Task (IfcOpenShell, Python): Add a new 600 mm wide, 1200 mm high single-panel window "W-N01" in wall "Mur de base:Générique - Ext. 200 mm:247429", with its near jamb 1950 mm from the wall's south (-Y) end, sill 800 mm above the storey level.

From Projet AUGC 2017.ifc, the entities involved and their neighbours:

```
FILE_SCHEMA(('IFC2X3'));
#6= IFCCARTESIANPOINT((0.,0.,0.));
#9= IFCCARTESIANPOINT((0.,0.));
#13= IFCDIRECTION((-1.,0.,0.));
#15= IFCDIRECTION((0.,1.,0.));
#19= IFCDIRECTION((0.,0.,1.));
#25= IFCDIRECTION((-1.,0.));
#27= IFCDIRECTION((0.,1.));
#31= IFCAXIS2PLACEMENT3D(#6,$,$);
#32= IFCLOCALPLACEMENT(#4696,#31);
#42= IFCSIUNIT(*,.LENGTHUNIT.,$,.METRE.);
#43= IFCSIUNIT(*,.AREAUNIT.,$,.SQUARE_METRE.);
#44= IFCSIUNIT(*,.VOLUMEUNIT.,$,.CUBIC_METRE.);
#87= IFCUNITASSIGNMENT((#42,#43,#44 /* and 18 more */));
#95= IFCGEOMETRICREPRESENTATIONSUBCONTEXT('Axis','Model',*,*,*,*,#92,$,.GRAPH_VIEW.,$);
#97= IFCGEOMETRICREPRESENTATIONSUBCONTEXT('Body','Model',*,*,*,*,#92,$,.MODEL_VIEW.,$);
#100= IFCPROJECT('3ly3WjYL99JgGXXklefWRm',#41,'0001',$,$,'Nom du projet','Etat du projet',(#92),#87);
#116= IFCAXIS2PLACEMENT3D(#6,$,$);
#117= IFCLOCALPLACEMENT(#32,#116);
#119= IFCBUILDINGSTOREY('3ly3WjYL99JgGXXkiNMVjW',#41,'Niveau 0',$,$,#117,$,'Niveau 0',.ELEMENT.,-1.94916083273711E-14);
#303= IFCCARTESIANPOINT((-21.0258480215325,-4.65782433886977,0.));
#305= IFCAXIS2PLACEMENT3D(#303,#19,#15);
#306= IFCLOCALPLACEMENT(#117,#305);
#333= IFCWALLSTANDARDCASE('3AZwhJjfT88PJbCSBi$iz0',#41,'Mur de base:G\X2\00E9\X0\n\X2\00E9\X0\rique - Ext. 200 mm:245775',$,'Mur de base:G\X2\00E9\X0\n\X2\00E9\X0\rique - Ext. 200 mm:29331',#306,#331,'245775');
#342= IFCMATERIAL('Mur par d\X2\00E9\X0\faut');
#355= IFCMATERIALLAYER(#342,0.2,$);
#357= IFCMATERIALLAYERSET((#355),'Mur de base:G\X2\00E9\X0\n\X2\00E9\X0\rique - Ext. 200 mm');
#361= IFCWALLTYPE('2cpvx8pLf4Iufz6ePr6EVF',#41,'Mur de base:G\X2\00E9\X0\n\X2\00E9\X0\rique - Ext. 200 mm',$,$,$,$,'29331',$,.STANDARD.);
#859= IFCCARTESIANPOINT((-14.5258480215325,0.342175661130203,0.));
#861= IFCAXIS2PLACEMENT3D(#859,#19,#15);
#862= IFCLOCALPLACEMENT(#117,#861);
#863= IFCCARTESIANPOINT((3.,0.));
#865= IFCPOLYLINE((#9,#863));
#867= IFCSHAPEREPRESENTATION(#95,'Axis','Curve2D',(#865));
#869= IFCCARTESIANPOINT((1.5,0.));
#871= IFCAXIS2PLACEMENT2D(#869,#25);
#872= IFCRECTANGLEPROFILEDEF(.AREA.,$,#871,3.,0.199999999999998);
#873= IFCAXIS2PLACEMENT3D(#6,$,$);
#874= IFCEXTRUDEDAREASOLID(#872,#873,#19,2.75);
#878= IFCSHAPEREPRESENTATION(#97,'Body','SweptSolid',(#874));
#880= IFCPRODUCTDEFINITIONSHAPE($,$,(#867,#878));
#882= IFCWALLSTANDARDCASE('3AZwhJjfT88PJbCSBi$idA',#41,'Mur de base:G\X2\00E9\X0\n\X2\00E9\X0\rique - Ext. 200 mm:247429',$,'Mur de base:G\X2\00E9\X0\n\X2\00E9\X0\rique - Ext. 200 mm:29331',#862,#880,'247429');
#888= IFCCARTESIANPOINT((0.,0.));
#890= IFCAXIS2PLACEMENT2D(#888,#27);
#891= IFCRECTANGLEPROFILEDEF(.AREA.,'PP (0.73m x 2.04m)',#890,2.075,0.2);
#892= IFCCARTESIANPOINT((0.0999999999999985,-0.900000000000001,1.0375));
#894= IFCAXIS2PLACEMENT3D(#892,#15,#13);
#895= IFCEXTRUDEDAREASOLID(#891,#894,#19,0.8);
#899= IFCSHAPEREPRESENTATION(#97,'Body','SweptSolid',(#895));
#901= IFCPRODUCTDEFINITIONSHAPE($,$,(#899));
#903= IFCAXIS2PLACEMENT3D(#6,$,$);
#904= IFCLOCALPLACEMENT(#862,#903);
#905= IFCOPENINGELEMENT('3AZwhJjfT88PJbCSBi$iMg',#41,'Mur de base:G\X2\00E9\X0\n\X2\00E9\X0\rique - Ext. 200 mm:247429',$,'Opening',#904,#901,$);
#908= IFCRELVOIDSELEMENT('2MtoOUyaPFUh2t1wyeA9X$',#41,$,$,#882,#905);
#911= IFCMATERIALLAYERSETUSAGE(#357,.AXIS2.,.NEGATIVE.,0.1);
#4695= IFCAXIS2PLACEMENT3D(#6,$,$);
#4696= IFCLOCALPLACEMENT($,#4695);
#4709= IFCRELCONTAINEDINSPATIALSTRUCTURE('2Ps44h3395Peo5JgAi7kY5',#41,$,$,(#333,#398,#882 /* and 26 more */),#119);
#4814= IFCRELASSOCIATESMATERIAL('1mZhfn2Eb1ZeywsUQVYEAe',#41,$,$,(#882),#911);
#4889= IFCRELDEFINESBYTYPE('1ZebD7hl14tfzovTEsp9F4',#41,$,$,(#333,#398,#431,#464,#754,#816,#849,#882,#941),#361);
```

```python
import numpy as np
import ifcopenshell
import ifcopenshell.api.feature
import ifcopenshell.api.geometry
import ifcopenshell.api.root
import ifcopenshell.api.spatial
import ifcopenshell.api.type
import ifcopenshell.geom
import ifcopenshell.util.element
import ifcopenshell.util.placement
import ifcopenshell.util.representation
import ifcopenshell.util.shape
import ifcopenshell.util.unit

model = ifcopenshell.open("Projet AUGC 2017.ifc")
unit_scale = ifcopenshell.util.unit.calculate_unit_scale(model)
settings = ifcopenshell.geom.settings()


def volume(element):
    """Net volume in cubic metres, openings subtracted."""
    shape = ifcopenshell.geom.create_shape(settings, element)
    return ifcopenshell.util.shape.get_volume(shape.geometry)


wall = model.by_guid("3AZwhJjfT88PJbCSBi$idA")
storey = ifcopenshell.util.element.get_container(wall, ifc_class="IfcBuildingStorey")
context = ifcopenshell.util.representation.get_context(model, "Model", "Body", "MODEL_VIEW")
before = volume(wall)

width, height, from_end, sill = 0.6, 1.2, 1.95, 0.8  # metres

# The wall runs along its own X axis, and the end named is its -X end.
wall_shape = ifcopenshell.geom.create_shape(settings, wall)
x, y, z = ifcopenshell.util.shape.get_vertices(wall_shape.geometry).T
start = x.min() + from_end
face, thickness = float(y.min()), float(y.max() - y.min())
wall_matrix = ifcopenshell.util.placement.get_local_placement(wall.ObjectPlacement)
level = ifcopenshell.util.placement.get_local_placement(storey.ObjectPlacement)[2, 3]


def in_wall(x, y):
    """Placement at x, y metres in the wall's axes, at sill height."""
    matrix = wall_matrix.copy()
    matrix[:, 3] = wall_matrix @ np.array([x / unit_scale, y / unit_scale, 0.0, 1.0])
    matrix[2, 3] = level + sill / unit_scale
    return matrix


# Opening: a box that overshoots both wall faces by 50 mm.
opening = ifcopenshell.api.root.create_entity(model, ifc_class="IfcOpeningElement")
box = ifcopenshell.api.geometry.add_wall_representation(
    model, context=context, length=width, height=height, thickness=thickness + 0.1
)
ifcopenshell.api.geometry.assign_representation(model, product=opening, representation=box)
ifcopenshell.api.geometry.edit_object_placement(model, product=opening, matrix=in_wall(start, face - 0.05), is_si=False)
ifcopenshell.api.feature.add_feature(model, feature=opening, element=wall)

window = ifcopenshell.api.root.create_entity(model, ifc_class="IfcWindow", name="W-N01")
window.OverallWidth, window.OverallHeight = width / unit_scale, height / unit_scale
body = ifcopenshell.api.geometry.add_window_representation(
    model,
    context=context,
    overall_width=window.OverallWidth,
    overall_height=window.OverallHeight,
    partition_type="SINGLE_PANEL",
)
ifcopenshell.api.geometry.assign_representation(model, product=window, representation=body)
ifcopenshell.api.spatial.assign_container(model, products=[window], relating_structure=storey)
fills = ifcopenshell.api.feature.add_filling(model, opening=opening, element=window)
fills.OwnerHistory = window.OwnerHistory  # required in IFC2X3

# IFC2X3 keeps the operation on the window style.
style = ifcopenshell.api.root.create_entity(model, ifc_class="IfcWindowStyle", name="W-N01")
style.OperationType, style.ConstructionType = "SINGLE_PANEL", "NOTDEFINED"
style.ParameterTakesPrecedence = style.Sizeable = False
ifcopenshell.api.type.assign_type(model, related_objects=[window], relating_type=style)

# Centre the window in the wall's thickness.
ifcopenshell.api.geometry.edit_object_placement(model, product=window, matrix=in_wall(start, face), is_si=False)
window_shape = ifcopenshell.geom.create_shape(settings, window)
depth = ifcopenshell.util.shape.get_vertices(window_shape.geometry)[:, 1]
offset = face + thickness / 2 - (depth.min() + depth.max()) / 2
ifcopenshell.api.geometry.edit_object_placement(model, product=window, matrix=in_wall(start, offset), is_si=False)

after = volume(wall)

print(f"wall volume {before:.3f} -> {after:.3f} m3")

model.write("Projet AUGC 2017_rev.ifc")
```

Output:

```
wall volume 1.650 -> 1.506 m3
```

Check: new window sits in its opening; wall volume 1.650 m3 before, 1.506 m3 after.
